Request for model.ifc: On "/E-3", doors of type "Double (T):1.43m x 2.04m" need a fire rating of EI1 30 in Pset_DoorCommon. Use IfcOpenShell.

First a look at what the model holds.

```python
import ifcopenshell
import ifcopenshell.util.element

model = ifcopenshell.open("model.ifc")
print(model.schema)
storey = next(s for s in model.by_type("IfcBuildingStorey") if s.Name == "/E-3")
doors = [e for e in ifcopenshell.util.element.get_decomposition(storey) if e.is_a("IfcDoor")]
seen = {}
for e in doors:
    element_type = ifcopenshell.util.element.get_type(e)
    key = (element_type.Name if element_type != e and element_type else None, ifcopenshell.util.element.get_pset(e, "Pset_DoorCommon", "FireRating"))
    seen[key] = seen.get(key, 0) + 1
for (name, value), count in sorted(seen.items(), key=str):
    print(count, "x", name, "|", value)
```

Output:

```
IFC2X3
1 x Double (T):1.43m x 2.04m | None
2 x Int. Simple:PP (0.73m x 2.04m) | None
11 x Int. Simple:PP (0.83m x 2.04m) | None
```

```python
import ifcopenshell
import ifcopenshell.api.pset
import ifcopenshell.util.element

model = ifcopenshell.open("model.ifc")

storey = next(s for s in model.by_type("IfcBuildingStorey") if s.Name == "/E-3")
doors = [e for e in ifcopenshell.util.element.get_decomposition(storey) if e.is_a("IfcDoor")]

count = 0
for e in doors:
    element_type = ifcopenshell.util.element.get_type(e)
    if element_type in (None, e) or element_type.Name != "Double (T):1.43m x 2.04m":
        continue
    # add_pset returns the element's existing set when there is one.
    pset = ifcopenshell.api.pset.add_pset(model, product=e, name="Pset_DoorCommon")
    ifcopenshell.api.pset.edit_pset(model, pset=pset, properties={"FireRating": "EI1 30"})
    count += 1

print(count, "doors updated")

model.write("model_v2.ifc")
```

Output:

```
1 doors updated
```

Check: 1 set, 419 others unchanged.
